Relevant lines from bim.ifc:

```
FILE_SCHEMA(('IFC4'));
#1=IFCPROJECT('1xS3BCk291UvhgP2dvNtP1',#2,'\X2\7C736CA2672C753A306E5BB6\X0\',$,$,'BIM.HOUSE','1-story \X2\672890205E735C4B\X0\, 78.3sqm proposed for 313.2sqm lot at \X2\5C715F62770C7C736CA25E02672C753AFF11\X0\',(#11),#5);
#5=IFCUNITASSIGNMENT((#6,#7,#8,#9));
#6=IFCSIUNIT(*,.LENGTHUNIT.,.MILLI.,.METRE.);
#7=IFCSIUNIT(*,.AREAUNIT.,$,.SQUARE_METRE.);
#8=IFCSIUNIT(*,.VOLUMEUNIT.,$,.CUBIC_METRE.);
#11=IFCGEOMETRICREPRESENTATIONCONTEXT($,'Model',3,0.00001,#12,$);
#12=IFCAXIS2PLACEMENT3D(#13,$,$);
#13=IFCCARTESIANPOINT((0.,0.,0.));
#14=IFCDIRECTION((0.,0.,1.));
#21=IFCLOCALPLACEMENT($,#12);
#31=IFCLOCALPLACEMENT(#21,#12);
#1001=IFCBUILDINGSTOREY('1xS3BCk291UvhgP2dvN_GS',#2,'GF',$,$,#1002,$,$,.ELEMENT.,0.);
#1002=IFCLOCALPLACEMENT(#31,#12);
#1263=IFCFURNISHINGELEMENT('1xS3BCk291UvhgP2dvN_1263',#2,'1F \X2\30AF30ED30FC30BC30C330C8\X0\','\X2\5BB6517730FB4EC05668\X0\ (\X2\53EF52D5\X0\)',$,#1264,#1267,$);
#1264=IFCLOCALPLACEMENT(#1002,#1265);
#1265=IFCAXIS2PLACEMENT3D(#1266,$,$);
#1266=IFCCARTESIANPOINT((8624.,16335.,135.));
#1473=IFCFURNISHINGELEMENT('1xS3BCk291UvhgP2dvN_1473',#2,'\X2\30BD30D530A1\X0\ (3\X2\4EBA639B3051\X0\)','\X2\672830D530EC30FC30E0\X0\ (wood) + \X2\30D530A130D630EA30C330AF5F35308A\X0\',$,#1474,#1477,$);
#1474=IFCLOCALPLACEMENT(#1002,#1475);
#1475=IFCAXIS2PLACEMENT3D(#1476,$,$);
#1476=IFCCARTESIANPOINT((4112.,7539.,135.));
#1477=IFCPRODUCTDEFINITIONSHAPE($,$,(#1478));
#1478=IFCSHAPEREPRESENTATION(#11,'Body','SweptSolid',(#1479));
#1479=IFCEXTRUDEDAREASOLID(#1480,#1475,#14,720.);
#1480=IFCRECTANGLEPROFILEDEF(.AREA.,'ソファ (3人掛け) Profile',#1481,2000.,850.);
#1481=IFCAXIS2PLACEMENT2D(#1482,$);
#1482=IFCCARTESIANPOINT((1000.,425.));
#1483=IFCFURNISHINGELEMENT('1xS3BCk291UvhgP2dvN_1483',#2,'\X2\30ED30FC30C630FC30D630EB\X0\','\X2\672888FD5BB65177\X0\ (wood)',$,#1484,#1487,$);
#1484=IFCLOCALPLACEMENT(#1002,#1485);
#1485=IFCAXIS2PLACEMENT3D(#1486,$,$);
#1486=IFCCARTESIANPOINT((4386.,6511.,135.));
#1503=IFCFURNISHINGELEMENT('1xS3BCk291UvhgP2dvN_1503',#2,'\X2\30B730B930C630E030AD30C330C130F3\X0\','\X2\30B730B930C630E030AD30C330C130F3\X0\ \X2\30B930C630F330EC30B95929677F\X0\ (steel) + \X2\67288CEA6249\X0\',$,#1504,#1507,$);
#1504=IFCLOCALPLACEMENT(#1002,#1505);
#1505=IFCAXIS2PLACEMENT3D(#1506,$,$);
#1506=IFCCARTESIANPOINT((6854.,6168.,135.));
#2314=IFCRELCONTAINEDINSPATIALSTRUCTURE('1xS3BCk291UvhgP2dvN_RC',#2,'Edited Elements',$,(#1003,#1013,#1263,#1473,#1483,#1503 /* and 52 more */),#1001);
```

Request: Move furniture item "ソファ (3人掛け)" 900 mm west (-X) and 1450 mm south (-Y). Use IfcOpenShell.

```python
import ifcopenshell
import ifcopenshell.api.geometry
import ifcopenshell.util.placement

model = ifcopenshell.open("bim.ifc")

item = model.by_guid("1xS3BCk291UvhgP2dvN_1473")
matrix = ifcopenshell.util.placement.get_local_placement(item.ObjectPlacement)
matrix[0, 3] -= 900.0
matrix[1, 3] -= 1450.0
ifcopenshell.api.geometry.edit_object_placement(model, product=item, matrix=matrix, is_si=False)

print(ifcopenshell.util.placement.get_local_placement(item.ObjectPlacement).round(3) + 0.0)

model.write("bim_edited.ifc")
```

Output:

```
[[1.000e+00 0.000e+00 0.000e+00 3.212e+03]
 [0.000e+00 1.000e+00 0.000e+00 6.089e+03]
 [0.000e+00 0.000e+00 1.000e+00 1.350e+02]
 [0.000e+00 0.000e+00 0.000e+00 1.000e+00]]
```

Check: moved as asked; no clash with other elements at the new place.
